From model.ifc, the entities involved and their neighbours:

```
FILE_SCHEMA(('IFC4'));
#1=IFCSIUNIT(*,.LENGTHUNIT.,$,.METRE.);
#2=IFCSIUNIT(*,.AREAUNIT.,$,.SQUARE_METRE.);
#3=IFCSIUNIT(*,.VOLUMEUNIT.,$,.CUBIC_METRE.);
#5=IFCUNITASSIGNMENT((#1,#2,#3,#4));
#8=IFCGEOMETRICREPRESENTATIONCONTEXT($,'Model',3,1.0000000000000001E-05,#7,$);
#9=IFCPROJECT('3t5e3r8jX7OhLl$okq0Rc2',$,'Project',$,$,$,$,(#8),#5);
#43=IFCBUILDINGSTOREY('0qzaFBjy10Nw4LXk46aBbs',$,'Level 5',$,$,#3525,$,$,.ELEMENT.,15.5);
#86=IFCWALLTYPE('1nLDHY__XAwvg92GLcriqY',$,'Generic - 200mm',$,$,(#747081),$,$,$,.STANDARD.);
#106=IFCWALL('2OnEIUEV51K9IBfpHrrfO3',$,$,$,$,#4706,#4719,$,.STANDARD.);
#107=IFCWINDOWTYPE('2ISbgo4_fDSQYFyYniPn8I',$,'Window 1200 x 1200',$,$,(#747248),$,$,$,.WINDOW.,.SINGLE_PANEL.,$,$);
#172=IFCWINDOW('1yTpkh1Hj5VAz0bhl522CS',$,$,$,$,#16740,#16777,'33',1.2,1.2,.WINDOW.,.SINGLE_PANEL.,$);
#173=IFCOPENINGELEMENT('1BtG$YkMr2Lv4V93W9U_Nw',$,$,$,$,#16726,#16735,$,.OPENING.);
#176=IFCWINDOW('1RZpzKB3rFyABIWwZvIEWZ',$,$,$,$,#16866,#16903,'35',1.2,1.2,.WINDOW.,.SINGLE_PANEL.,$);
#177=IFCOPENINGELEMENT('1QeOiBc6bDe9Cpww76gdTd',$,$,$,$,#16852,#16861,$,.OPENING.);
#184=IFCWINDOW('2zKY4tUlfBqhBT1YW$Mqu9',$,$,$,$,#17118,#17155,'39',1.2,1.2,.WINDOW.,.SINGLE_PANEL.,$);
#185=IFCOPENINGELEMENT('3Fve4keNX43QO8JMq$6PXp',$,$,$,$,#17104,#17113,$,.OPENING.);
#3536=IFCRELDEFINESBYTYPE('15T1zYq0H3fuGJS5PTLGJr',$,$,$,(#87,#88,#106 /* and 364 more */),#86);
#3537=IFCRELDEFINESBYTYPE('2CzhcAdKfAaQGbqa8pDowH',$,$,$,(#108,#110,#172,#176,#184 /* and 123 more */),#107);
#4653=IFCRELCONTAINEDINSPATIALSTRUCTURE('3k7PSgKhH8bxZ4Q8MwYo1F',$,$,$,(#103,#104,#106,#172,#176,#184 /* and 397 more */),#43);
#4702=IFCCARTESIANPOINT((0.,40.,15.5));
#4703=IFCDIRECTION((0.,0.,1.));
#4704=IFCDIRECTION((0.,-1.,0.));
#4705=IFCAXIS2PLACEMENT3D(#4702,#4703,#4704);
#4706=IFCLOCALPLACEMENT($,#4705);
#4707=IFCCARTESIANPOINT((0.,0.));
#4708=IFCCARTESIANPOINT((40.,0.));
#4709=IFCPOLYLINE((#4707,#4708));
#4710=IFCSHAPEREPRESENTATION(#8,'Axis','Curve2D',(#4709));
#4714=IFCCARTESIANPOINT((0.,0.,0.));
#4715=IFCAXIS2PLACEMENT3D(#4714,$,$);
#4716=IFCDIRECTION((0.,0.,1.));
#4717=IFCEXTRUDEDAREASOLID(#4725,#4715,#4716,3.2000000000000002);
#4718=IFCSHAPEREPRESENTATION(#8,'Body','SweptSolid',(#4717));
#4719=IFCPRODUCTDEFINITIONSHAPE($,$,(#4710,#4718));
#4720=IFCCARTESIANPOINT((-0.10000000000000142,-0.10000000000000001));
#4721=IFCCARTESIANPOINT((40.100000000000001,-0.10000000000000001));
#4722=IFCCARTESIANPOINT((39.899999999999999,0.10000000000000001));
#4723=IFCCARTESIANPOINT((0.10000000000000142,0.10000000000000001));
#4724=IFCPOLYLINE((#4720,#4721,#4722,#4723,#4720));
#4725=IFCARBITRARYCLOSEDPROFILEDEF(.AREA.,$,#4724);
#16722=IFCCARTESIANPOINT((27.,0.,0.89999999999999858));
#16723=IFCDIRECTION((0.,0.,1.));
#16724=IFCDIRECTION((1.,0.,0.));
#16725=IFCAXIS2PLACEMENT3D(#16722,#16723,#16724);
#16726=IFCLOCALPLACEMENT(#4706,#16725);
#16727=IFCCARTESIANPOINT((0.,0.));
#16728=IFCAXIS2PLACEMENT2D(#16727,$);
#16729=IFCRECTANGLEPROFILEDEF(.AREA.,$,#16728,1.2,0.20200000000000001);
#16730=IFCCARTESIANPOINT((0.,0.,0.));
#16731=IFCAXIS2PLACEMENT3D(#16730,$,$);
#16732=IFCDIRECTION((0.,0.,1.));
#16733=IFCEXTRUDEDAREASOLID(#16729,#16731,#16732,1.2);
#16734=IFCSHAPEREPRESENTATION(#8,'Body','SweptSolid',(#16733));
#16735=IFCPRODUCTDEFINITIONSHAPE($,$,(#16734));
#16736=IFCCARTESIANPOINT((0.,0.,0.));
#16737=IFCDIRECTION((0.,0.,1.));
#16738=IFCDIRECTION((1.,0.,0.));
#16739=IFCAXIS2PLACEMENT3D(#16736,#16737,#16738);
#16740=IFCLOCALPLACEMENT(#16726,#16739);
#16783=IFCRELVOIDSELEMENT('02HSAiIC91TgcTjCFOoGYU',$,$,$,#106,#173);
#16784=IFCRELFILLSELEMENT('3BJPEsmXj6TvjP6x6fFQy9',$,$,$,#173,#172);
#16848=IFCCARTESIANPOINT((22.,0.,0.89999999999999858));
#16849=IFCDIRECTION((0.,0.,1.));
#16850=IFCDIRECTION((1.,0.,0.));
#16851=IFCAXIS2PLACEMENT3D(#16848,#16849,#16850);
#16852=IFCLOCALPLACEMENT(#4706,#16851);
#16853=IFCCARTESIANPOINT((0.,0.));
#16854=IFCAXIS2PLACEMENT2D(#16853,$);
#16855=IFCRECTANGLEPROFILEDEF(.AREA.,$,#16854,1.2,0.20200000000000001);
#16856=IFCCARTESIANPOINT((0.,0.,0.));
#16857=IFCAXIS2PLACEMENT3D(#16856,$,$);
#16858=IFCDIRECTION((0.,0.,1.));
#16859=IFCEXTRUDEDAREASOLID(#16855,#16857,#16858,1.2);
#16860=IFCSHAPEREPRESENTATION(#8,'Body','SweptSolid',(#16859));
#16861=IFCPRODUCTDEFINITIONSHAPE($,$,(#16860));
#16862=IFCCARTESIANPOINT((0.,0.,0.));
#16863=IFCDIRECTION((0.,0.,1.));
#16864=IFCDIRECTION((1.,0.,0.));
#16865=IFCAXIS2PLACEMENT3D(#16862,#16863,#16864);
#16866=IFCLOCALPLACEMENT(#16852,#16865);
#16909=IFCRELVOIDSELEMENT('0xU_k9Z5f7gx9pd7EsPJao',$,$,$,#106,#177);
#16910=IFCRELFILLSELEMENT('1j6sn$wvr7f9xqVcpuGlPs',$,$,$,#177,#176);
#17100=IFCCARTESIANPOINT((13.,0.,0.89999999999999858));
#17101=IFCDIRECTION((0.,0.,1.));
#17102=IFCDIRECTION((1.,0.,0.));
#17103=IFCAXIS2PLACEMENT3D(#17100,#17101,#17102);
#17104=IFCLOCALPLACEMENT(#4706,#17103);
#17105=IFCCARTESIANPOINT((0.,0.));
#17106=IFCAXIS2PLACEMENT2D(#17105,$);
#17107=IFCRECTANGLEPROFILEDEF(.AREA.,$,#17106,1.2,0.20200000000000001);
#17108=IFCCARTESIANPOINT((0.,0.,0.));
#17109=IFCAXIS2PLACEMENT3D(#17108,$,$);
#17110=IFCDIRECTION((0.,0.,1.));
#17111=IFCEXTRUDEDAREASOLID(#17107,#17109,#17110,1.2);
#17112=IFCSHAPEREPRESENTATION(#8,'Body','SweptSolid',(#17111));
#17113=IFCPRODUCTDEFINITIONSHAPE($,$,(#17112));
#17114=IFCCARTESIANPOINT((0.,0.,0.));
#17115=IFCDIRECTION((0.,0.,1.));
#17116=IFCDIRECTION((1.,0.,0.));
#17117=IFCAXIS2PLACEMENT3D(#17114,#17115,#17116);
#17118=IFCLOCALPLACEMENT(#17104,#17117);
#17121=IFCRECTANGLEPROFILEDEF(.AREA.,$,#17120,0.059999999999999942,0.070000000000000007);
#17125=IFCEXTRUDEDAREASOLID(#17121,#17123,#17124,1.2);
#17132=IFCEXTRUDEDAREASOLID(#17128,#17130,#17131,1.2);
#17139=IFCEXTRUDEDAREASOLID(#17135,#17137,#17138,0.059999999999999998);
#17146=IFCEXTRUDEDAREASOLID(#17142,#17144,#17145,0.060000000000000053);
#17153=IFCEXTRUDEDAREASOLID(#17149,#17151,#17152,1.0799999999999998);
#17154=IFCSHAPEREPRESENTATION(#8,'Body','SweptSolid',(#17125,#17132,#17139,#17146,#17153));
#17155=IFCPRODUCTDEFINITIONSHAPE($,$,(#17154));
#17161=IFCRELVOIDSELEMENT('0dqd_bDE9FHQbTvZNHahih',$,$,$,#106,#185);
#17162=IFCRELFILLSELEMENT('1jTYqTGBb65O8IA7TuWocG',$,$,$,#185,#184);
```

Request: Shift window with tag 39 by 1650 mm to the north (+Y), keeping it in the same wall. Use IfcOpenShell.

```python
import ifcopenshell
import ifcopenshell.api.geometry
import ifcopenshell.util.placement

model = ifcopenshell.open("model.ifc")

window = model.by_id(184)
opening = window.FillsVoids[0].RelatingOpeningElement
wall = opening.VoidsElements[0].RelatingBuildingElement

wall_matrix = ifcopenshell.util.placement.get_local_placement(wall.ObjectPlacement)
shift = wall_matrix[:3, 0] * -1.65
before = ifcopenshell.util.placement.get_local_placement(window.ObjectPlacement)[:3, 3].copy()

# The window is placed relative to its opening, so it follows when the opening moves.
matrix = ifcopenshell.util.placement.get_local_placement(opening.ObjectPlacement)
matrix[:3, 3] += shift
ifcopenshell.api.geometry.edit_object_placement(
    model, product=opening, matrix=matrix, is_si=False, should_transform_children=True
)

after = ifcopenshell.util.placement.get_local_placement(window.ObjectPlacement)[:3, 3]
print("window moved by", (after - before).round(3) + 0.0)

model.write("model_updated.ifc")
```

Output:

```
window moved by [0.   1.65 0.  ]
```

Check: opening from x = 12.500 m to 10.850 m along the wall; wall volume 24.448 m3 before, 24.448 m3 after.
